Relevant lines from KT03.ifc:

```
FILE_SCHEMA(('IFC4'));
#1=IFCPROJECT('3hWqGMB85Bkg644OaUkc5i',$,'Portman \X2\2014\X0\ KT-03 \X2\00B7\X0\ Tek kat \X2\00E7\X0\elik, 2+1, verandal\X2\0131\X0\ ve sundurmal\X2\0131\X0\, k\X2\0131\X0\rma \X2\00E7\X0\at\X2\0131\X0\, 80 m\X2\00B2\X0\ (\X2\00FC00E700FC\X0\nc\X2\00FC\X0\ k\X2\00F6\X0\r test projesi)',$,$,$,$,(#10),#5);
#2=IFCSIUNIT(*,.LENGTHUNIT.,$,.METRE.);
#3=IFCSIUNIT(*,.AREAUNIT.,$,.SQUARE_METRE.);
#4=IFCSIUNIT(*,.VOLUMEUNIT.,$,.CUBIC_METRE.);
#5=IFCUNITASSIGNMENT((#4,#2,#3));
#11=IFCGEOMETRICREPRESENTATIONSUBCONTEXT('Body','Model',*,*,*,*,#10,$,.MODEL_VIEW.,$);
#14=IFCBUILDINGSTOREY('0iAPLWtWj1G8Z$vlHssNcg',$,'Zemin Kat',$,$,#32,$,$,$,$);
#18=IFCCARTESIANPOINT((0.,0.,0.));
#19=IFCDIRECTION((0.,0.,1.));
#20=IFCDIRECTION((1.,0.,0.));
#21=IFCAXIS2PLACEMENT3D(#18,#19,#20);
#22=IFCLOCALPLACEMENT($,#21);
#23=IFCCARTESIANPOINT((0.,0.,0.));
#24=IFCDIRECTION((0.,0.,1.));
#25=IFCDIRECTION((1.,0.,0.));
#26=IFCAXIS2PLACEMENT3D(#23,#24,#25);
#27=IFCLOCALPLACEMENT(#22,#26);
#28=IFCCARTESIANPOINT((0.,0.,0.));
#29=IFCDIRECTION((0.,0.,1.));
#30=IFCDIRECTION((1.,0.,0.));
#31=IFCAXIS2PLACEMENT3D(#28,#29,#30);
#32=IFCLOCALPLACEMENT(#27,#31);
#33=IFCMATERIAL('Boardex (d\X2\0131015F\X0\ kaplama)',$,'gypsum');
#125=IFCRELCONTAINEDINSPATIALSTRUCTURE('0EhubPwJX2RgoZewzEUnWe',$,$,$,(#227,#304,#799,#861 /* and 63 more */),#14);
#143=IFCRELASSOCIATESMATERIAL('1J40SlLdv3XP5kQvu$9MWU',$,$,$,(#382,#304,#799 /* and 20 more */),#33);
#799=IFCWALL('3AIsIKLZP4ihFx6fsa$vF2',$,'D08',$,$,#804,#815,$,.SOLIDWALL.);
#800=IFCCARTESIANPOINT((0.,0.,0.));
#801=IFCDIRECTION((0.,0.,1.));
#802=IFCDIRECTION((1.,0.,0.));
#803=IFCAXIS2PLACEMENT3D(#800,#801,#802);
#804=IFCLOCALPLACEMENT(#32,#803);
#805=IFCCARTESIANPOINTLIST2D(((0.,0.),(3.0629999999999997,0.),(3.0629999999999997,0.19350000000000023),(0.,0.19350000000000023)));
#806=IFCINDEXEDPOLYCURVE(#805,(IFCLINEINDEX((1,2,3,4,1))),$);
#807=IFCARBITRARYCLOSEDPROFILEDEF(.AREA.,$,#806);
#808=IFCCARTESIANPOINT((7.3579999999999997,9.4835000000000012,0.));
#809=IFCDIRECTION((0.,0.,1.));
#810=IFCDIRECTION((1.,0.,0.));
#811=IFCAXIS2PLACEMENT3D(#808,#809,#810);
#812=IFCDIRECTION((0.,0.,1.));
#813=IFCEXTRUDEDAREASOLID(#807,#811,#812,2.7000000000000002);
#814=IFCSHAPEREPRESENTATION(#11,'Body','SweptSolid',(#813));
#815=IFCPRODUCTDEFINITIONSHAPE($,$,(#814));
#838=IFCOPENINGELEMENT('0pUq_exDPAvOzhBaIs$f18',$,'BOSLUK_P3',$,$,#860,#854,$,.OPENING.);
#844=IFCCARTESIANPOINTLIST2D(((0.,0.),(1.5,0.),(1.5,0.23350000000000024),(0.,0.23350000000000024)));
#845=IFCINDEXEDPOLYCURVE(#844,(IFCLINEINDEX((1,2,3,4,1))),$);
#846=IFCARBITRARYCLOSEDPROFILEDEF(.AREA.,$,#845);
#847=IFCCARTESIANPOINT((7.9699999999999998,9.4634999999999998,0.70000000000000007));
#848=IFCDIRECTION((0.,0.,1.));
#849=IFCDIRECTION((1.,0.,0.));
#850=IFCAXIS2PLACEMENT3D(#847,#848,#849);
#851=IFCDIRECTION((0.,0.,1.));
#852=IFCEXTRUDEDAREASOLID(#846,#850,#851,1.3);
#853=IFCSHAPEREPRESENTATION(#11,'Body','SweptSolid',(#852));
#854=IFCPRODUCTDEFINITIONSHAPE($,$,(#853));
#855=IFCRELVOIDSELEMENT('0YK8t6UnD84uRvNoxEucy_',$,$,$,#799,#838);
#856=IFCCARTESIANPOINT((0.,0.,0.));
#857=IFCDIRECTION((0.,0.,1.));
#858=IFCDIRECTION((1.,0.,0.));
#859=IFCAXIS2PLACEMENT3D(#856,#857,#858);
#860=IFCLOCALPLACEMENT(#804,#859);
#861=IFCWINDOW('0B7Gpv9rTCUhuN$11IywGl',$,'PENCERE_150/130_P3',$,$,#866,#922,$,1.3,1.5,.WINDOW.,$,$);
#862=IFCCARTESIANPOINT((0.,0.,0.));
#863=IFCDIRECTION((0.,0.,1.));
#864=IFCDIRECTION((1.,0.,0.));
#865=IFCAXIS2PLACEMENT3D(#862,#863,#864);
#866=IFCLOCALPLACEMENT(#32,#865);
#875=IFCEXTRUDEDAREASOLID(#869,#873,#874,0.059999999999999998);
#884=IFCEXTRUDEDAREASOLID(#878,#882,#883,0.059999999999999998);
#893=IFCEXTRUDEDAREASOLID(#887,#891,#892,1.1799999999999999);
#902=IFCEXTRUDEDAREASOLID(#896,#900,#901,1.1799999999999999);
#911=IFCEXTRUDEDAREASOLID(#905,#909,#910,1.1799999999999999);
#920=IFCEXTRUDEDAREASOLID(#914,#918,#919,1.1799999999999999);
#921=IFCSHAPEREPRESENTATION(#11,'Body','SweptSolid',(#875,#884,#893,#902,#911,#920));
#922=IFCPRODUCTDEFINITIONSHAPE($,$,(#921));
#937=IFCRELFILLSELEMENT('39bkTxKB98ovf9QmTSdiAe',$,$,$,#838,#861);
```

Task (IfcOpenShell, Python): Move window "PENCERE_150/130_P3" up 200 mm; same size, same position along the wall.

```python
import numpy as np
import ifcopenshell
import ifcopenshell.api.geometry
import ifcopenshell.util.placement
import ifcopenshell.util.unit

model = ifcopenshell.open("KT03.ifc")
unit_scale = ifcopenshell.util.unit.calculate_unit_scale(model)

window = model.by_guid("0B7Gpv9rTCUhuN$11IywGl")
opening = window.FillsVoids[0].RelatingOpeningElement
dz = 0.2

shift = np.array([0.0, 0.0, dz])
# The window is not placed relative to its opening, so move both.
for product in (opening, window):
    matrix = ifcopenshell.util.placement.get_local_placement(product.ObjectPlacement)
    matrix[:3, 3] += shift
    ifcopenshell.api.geometry.edit_object_placement(model, product=product, matrix=matrix, is_si=False)

print(f"moved by {dz * unit_scale:+.3f} m")

model.write("KT03_rev.ifc")
```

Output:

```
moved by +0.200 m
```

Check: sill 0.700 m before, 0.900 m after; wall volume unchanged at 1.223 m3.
